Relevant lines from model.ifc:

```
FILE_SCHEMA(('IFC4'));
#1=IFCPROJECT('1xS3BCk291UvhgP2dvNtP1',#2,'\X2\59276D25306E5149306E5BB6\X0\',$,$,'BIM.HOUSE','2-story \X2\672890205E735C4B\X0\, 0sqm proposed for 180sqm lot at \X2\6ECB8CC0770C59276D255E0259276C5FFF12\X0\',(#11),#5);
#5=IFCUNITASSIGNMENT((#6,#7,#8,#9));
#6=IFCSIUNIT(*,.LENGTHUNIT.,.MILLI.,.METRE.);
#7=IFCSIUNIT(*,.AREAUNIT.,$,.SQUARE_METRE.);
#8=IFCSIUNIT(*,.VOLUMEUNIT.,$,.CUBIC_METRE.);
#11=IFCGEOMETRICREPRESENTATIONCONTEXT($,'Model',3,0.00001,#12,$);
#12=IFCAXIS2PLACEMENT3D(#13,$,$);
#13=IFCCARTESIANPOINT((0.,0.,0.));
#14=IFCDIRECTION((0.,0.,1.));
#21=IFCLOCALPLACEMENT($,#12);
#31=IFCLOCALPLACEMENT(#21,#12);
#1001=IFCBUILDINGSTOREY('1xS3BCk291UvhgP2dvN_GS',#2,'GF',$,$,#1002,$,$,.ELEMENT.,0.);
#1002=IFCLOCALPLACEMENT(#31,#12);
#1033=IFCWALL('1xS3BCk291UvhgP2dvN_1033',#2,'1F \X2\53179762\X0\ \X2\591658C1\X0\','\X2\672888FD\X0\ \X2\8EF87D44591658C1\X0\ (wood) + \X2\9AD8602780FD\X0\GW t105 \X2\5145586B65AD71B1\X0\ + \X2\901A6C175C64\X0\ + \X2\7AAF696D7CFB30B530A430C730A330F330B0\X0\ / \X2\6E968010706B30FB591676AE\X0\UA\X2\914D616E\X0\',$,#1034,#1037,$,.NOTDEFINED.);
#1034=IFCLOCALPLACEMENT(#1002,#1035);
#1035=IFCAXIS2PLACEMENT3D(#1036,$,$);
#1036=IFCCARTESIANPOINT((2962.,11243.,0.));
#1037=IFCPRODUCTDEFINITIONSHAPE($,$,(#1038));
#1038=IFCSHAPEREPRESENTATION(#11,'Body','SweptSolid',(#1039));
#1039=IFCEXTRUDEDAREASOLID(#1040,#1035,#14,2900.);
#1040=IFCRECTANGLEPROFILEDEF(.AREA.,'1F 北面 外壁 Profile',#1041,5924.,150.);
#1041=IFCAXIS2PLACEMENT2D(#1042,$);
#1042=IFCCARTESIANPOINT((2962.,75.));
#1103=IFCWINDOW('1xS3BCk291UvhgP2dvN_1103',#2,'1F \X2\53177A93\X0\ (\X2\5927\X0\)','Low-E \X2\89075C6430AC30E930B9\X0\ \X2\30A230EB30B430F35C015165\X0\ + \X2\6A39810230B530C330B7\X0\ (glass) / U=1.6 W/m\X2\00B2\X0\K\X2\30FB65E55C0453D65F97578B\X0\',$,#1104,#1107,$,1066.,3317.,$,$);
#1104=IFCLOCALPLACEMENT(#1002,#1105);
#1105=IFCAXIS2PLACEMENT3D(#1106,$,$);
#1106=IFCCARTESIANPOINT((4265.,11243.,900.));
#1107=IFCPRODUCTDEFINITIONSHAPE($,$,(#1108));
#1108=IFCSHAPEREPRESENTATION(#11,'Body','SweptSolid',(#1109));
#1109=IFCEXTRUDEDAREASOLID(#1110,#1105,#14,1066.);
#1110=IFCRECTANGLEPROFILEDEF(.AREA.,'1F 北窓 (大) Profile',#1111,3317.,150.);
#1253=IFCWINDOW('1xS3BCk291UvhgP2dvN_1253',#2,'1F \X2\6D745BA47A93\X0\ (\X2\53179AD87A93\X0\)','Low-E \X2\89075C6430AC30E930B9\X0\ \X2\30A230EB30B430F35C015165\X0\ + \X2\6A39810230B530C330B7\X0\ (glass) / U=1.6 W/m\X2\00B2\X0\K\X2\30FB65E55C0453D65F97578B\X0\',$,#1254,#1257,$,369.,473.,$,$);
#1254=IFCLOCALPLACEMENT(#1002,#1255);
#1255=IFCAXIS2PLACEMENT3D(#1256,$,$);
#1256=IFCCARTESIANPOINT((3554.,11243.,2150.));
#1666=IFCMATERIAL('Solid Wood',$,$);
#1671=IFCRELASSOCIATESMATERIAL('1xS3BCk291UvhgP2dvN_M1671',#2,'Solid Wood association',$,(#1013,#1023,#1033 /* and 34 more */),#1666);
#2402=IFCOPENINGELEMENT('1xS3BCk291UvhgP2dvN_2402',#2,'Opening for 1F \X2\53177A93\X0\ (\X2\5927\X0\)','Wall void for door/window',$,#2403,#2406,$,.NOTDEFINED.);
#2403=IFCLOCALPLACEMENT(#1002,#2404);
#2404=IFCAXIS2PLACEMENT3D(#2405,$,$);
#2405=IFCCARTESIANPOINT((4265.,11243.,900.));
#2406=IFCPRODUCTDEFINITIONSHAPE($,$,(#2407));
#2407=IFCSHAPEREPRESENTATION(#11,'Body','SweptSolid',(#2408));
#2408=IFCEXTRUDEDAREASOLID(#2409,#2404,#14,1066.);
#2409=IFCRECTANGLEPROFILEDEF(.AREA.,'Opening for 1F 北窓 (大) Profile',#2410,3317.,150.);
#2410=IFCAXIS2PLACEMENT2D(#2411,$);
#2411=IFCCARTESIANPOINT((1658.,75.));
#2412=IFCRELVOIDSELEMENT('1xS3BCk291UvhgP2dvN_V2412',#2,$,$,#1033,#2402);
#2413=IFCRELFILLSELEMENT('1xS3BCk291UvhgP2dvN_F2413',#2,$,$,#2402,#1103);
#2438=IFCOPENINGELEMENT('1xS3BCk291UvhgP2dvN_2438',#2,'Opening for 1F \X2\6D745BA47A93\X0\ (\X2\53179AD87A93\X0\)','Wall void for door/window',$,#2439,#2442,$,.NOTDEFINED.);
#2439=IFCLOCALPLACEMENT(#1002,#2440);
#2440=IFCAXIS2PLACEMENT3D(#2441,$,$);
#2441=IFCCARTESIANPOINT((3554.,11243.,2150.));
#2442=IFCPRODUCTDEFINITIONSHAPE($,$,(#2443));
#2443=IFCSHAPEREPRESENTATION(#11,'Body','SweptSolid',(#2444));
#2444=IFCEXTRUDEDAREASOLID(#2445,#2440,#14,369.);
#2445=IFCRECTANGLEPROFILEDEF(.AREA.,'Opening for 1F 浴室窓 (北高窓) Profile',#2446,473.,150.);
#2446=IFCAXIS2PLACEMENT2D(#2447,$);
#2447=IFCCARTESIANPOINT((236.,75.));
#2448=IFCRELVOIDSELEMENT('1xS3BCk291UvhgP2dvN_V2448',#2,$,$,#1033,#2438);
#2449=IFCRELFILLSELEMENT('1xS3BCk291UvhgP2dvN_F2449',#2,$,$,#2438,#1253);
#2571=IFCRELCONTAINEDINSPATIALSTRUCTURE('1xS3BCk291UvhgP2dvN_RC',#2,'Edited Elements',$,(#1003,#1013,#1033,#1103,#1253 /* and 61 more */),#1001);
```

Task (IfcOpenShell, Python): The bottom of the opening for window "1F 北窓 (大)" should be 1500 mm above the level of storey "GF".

```python
import numpy as np
import ifcopenshell
import ifcopenshell.api.geometry
import ifcopenshell.geom
import ifcopenshell.util.element
import ifcopenshell.util.placement
import ifcopenshell.util.shape
import ifcopenshell.util.unit

model = ifcopenshell.open("model.ifc")
unit_scale = ifcopenshell.util.unit.calculate_unit_scale(model)

window = model.by_guid("1xS3BCk291UvhgP2dvN_1103")
opening = window.FillsVoids[0].RelatingOpeningElement
storey = ifcopenshell.util.element.get_container(window, ifc_class="IfcBuildingStorey")
level = ifcopenshell.util.placement.get_local_placement(storey.ObjectPlacement)[2, 3]

# The opening's origin need not be at the sill, so measure its lowest point.
shape = ifcopenshell.geom.create_shape(ifcopenshell.geom.settings(), opening)
bottom = ifcopenshell.util.shape.get_shape_bottom_elevation(shape, shape.geometry) / unit_scale
dz = level + 1.5 / unit_scale - bottom

shift = np.array([0.0, 0.0, dz])
# The window is not placed relative to its opening, so move both.
for product in (opening, window):
    matrix = ifcopenshell.util.placement.get_local_placement(product.ObjectPlacement)
    matrix[:3, 3] += shift
    ifcopenshell.api.geometry.edit_object_placement(model, product=product, matrix=matrix, is_si=False)

print(f"moved by {dz * unit_scale:+.3f} m")

model.write("model_updated.ifc")
```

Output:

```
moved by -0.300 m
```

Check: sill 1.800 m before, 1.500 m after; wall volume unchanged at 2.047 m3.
